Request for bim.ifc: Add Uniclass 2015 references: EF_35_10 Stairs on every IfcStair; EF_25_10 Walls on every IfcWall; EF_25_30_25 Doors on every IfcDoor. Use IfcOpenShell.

First a look at what the model holds.

```python
import ifcopenshell

model = ifcopenshell.open("bim.ifc")
print(model.schema)
print("classifications:", [c.Name for c in model.by_type("IfcClassification")])
for ifc_class in ("IfcDoor", "IfcRoof", "IfcStair", "IfcWall", "IfcWindow"):
    print(ifc_class, len(model.by_type(ifc_class)))
```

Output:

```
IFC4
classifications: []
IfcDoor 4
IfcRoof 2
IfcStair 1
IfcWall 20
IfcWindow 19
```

```python
import ifcopenshell
import ifcopenshell.api.classification

model = ifcopenshell.open("bim.ifc")

system = ifcopenshell.api.classification.add_classification(model, classification="Uniclass 2015")

codes = {
    "IfcStair": ("EF_35_10", "Stairs"),
    "IfcWall": ("EF_25_10", "Walls"),
    "IfcDoor": ("EF_25_30_25", "Doors"),
}
for ifc_class, (code, name) in codes.items():
    products = model.by_type(ifc_class)
    ifcopenshell.api.classification.add_reference(
        model, products=products, classification=system, identification=code, name=name
    )
    print(code, len(products))

model.write("bim_edited.ifc")
```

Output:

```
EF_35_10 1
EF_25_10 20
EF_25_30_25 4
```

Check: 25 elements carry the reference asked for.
